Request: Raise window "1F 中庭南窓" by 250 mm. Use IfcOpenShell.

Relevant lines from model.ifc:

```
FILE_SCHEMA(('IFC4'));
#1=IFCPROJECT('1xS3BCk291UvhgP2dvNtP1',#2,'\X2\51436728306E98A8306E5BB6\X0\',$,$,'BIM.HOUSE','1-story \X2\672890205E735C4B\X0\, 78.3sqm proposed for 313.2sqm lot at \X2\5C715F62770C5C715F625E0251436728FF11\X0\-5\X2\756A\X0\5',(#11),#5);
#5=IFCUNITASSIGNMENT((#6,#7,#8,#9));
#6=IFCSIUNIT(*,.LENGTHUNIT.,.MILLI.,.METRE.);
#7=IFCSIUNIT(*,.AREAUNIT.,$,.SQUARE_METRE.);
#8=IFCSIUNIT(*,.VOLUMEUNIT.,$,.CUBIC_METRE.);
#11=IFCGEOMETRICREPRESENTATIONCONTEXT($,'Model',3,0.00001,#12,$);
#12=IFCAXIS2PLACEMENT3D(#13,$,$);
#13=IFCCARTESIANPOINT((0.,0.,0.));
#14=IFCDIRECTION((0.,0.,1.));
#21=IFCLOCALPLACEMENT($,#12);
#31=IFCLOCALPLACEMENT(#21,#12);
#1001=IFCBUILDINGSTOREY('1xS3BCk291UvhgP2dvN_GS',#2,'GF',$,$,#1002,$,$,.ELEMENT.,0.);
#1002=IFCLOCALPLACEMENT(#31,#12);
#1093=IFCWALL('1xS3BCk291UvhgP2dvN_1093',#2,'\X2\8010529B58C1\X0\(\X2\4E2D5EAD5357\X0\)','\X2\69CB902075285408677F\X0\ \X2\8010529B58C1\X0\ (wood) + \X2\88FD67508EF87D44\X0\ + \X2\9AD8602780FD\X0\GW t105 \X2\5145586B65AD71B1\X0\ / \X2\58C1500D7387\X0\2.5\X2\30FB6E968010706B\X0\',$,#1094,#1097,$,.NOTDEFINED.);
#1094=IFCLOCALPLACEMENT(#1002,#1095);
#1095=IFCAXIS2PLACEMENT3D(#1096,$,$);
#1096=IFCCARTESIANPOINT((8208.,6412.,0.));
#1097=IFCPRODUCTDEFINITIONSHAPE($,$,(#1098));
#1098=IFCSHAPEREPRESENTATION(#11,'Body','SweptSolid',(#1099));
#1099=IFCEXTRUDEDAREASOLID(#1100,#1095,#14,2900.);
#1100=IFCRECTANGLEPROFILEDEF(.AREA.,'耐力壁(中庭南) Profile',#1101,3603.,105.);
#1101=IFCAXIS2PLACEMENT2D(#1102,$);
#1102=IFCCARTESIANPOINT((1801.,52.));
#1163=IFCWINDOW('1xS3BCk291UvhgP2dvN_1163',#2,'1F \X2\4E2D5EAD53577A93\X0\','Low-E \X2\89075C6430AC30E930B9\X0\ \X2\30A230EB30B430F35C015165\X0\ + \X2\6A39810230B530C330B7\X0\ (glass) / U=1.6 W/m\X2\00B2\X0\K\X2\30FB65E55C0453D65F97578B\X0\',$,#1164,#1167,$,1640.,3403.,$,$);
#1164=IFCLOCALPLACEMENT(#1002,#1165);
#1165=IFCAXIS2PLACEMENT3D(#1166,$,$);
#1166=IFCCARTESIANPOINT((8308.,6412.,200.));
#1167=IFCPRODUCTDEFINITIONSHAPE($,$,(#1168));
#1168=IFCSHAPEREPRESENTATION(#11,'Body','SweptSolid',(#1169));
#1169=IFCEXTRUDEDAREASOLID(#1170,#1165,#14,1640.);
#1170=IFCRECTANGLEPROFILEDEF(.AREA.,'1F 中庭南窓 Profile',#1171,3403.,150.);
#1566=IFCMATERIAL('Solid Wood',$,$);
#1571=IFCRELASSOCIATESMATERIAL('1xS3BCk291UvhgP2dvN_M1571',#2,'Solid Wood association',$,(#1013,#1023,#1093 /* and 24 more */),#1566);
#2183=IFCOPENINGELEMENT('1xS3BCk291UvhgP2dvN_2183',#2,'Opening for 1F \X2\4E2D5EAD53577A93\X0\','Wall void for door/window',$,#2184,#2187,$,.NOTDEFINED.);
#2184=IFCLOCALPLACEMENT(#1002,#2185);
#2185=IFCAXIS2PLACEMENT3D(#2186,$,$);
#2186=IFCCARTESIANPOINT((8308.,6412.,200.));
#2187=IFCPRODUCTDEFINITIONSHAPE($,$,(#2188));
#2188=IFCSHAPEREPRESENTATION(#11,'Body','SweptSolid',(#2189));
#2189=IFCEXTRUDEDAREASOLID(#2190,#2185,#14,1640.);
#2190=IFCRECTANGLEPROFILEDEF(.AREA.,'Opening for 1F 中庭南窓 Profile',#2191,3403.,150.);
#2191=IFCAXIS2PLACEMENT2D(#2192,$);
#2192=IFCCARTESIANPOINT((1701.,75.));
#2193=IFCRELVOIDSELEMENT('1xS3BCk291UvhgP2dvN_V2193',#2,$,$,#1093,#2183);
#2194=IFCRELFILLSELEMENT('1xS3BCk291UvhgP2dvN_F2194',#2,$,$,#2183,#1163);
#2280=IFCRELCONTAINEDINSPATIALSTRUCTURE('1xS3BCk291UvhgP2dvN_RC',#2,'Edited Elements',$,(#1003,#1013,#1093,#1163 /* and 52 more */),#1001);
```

```python
import numpy as np
import ifcopenshell
import ifcopenshell.api.geometry
import ifcopenshell.util.placement
import ifcopenshell.util.unit

model = ifcopenshell.open("model.ifc")
unit_scale = ifcopenshell.util.unit.calculate_unit_scale(model)

window = model.by_id(1163)
opening = window.FillsVoids[0].RelatingOpeningElement
dz = 0.25 / unit_scale

shift = np.array([0.0, 0.0, dz])
# The window is not placed relative to its opening, so move both.
for product in (opening, window):
    matrix = ifcopenshell.util.placement.get_local_placement(product.ObjectPlacement)
    matrix[:3, 3] += shift
    ifcopenshell.api.geometry.edit_object_placement(model, product=product, matrix=matrix, is_si=False)

print(f"moved by {dz * unit_scale:+.3f} m")

model.write("model-out.ifc")
```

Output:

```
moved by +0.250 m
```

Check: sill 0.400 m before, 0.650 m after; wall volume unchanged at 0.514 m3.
